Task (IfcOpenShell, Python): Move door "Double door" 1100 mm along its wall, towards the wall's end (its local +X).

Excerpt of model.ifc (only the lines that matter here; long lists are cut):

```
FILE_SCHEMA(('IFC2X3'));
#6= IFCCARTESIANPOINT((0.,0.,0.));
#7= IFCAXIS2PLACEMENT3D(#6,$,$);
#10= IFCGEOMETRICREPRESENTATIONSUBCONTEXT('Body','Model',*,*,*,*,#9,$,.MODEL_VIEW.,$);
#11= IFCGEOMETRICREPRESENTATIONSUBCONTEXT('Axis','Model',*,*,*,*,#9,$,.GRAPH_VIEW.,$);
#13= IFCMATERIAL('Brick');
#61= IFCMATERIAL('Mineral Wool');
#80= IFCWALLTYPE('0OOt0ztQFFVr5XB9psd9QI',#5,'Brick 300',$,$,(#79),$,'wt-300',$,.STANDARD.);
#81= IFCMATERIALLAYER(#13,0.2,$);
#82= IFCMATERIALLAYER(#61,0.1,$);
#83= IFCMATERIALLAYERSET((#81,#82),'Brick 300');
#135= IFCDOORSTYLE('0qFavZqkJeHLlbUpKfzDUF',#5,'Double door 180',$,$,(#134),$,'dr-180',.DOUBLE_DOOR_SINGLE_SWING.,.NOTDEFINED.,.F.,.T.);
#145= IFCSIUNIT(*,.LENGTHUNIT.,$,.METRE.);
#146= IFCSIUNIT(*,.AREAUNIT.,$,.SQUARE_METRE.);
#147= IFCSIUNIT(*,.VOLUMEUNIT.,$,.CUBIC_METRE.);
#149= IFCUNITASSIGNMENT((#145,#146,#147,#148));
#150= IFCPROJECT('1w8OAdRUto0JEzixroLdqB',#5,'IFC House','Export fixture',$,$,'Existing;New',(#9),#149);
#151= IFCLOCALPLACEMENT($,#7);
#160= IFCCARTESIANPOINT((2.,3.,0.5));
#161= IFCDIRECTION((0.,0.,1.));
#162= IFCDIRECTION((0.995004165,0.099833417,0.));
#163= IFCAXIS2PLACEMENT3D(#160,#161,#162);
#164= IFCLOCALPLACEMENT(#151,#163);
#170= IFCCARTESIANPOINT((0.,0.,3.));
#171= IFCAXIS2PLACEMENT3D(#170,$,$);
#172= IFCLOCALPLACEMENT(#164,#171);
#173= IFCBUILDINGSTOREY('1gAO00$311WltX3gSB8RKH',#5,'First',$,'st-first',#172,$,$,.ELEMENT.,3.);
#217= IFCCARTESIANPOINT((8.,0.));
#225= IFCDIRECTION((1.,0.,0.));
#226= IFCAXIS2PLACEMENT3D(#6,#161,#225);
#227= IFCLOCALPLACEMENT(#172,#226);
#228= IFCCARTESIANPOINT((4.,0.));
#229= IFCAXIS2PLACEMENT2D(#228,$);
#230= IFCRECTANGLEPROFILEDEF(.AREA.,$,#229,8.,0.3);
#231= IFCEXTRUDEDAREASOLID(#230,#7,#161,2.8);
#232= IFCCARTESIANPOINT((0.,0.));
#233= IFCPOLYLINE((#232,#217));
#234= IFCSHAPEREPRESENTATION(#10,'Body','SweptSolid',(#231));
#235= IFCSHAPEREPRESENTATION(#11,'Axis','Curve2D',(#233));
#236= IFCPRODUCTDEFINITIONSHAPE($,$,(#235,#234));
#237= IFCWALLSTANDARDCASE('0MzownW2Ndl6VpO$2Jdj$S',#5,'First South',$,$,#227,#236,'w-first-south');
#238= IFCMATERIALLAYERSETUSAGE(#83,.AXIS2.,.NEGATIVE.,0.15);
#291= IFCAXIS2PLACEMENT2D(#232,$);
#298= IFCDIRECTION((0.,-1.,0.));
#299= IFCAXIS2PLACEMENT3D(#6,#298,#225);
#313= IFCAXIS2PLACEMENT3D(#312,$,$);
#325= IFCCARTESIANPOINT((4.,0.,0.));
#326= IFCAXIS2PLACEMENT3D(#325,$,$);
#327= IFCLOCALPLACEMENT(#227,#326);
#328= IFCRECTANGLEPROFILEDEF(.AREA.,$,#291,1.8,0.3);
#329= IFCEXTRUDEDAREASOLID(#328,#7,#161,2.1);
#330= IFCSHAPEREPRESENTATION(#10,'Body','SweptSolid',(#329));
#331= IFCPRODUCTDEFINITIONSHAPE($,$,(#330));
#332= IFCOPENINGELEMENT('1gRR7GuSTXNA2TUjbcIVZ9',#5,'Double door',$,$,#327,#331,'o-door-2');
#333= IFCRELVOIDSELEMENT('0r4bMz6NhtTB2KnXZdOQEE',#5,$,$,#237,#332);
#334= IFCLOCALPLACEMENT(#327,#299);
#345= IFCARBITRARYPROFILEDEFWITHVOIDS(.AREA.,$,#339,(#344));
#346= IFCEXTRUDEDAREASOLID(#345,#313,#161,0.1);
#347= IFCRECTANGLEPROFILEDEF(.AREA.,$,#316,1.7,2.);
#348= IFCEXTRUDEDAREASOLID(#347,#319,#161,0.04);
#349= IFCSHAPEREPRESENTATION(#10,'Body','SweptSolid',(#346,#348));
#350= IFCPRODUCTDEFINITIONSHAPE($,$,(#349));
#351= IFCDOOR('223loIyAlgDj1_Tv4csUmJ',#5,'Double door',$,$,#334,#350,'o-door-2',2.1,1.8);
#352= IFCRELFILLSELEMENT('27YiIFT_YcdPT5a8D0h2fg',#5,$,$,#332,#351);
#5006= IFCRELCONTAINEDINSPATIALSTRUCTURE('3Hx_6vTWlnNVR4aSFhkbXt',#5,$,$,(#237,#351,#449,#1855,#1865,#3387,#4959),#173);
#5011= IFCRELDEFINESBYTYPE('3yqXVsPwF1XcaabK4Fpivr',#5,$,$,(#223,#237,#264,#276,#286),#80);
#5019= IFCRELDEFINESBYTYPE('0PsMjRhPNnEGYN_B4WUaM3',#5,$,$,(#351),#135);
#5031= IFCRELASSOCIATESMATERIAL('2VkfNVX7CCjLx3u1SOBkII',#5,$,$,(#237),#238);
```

```python
import ifcopenshell
import ifcopenshell.api.geometry
import ifcopenshell.util.placement
import ifcopenshell.util.unit

model = ifcopenshell.open("model.ifc")
unit_scale = ifcopenshell.util.unit.calculate_unit_scale(model)

door = model.by_id(351)
opening = door.FillsVoids[0].RelatingOpeningElement
wall = opening.VoidsElements[0].RelatingBuildingElement

wall_matrix = ifcopenshell.util.placement.get_local_placement(wall.ObjectPlacement)
shift = wall_matrix[:3, 0] * 1.1 / unit_scale
before = ifcopenshell.util.placement.get_local_placement(door.ObjectPlacement)[:3, 3].copy()

# The door is placed relative to its opening, so it follows when the opening moves.
matrix = ifcopenshell.util.placement.get_local_placement(opening.ObjectPlacement)
matrix[:3, 3] += shift
ifcopenshell.api.geometry.edit_object_placement(
    model, product=opening, matrix=matrix, is_si=False, should_transform_children=True
)

after = ifcopenshell.util.placement.get_local_placement(door.ObjectPlacement)[:3, 3]
print("door moved by", (after - before).round(3) + 0.0)

model.write("model_v2.ifc")
```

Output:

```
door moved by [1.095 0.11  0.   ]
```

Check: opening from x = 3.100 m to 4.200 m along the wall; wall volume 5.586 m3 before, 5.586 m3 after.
